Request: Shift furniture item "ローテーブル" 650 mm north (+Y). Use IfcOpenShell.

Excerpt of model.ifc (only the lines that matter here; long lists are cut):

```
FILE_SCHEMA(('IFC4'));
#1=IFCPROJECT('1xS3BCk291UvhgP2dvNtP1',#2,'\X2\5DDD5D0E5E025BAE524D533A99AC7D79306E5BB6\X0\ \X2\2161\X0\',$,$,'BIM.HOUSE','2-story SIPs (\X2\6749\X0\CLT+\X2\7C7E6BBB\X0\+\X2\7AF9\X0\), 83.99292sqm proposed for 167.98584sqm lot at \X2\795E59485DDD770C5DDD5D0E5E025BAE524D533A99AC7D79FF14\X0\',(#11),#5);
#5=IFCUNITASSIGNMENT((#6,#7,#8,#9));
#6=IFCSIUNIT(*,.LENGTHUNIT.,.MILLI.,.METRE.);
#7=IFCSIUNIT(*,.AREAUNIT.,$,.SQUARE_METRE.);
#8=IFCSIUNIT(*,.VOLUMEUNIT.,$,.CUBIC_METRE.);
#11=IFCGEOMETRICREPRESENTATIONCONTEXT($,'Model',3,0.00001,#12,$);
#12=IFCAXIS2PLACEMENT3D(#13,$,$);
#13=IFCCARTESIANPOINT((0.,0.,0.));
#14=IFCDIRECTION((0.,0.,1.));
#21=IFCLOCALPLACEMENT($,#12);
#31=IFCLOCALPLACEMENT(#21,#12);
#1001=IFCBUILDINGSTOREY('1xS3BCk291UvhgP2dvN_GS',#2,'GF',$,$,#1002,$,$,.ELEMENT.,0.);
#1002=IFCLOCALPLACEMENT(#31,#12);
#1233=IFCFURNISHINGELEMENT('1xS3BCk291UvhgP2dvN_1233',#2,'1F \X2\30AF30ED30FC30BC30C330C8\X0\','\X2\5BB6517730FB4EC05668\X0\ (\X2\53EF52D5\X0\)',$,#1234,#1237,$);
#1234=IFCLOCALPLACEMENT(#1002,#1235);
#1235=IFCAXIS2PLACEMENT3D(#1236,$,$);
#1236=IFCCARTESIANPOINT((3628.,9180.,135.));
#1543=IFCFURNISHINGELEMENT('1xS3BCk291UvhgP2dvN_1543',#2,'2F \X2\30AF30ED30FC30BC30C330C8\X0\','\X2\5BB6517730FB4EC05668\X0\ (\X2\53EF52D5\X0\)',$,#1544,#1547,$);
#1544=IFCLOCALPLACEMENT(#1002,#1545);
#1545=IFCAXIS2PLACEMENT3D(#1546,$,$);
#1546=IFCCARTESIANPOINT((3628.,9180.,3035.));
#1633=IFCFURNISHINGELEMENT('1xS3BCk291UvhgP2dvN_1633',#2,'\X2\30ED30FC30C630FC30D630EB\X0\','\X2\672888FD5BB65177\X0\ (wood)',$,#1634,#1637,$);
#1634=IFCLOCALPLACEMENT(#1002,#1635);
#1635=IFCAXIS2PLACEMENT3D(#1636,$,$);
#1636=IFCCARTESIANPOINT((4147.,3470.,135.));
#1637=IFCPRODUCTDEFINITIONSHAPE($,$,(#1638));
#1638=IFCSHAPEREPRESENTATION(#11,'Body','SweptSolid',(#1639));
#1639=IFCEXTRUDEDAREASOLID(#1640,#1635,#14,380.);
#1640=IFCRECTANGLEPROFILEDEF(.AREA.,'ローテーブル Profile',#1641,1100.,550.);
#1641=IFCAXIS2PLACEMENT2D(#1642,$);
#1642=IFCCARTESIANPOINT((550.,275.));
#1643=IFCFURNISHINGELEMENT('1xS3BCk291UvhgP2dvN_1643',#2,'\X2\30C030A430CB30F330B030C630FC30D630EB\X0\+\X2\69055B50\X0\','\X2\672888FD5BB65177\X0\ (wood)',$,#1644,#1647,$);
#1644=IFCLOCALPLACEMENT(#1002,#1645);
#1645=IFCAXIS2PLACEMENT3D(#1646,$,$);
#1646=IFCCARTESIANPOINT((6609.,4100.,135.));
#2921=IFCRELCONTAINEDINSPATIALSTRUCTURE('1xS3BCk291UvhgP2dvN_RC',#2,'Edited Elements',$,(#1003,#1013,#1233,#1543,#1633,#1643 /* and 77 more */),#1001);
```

```python
import ifcopenshell
import ifcopenshell.api.geometry
import ifcopenshell.util.placement
import ifcopenshell.util.unit

model = ifcopenshell.open("model.ifc")
unit_scale = ifcopenshell.util.unit.calculate_unit_scale(model)

item = model.by_guid("1xS3BCk291UvhgP2dvN_1633")
matrix = ifcopenshell.util.placement.get_local_placement(item.ObjectPlacement)
matrix[1, 3] += 0.65 / unit_scale
ifcopenshell.api.geometry.edit_object_placement(model, product=item, matrix=matrix, is_si=False)

print(ifcopenshell.util.placement.get_local_placement(item.ObjectPlacement).round(3) + 0.0)

model.write("model_v2.ifc")
```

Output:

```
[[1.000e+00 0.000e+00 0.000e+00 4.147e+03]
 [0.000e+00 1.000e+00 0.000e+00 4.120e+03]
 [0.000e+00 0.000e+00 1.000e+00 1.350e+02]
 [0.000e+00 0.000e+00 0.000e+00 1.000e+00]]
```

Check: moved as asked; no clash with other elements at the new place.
